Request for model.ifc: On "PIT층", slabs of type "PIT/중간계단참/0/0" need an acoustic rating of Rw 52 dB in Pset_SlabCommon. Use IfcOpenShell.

First a look at what the model holds.

```python
import ifcopenshell
import ifcopenshell.util.element

model = ifcopenshell.open("model.ifc")
print(model.schema)
storey = next(s for s in model.by_type("IfcBuildingStorey") if s.Name == "PIT층")
slabs = [e for e in ifcopenshell.util.element.get_decomposition(storey) if e.is_a("IfcSlab")]
seen = {}
for e in slabs:
    element_type = ifcopenshell.util.element.get_type(e)
    key = (element_type.Name if element_type != e and element_type else None, ifcopenshell.util.element.get_pset(e, "Pset_SlabCommon", "AcousticRating"))
    seen[key] = seen.get(key, 0) + 1
for (name, value), count in sorted(seen.items(), key=str):
    print(count, "x", name, "|", value)
```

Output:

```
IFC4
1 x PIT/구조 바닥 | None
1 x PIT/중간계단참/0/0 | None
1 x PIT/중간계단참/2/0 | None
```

```python
import ifcopenshell
import ifcopenshell.api.pset
import ifcopenshell.util.element

model = ifcopenshell.open("model.ifc")

storey = next(s for s in model.by_type("IfcBuildingStorey") if s.Name == "PIT층")
slabs = [e for e in ifcopenshell.util.element.get_decomposition(storey) if e.is_a("IfcSlab")]

count = 0
for e in slabs:
    element_type = ifcopenshell.util.element.get_type(e)
    if element_type in (None, e) or element_type.Name != "PIT/중간계단참/0/0":
        continue
    # add_pset returns the element's existing set when there is one.
    pset = ifcopenshell.api.pset.add_pset(model, product=e, name="Pset_SlabCommon")
    ifcopenshell.api.pset.edit_pset(model, pset=pset, properties={"AcousticRating": "Rw 52 dB"})
    count += 1

print(count, "slabs updated")

model.write("model-out.ifc")
```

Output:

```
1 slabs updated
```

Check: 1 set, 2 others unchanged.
